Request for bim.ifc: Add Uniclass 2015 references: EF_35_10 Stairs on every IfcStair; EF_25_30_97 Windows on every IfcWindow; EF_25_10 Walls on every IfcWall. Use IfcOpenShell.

First a look at what the model holds.

```python
import ifcopenshell

model = ifcopenshell.open("bim.ifc")
print(model.schema)
print("classifications:", [c.Name for c in model.by_type("IfcClassification")])
for ifc_class in ("IfcDoor", "IfcRoof", "IfcStair", "IfcWall", "IfcWindow"):
    print(ifc_class, len(model.by_type(ifc_class)))
```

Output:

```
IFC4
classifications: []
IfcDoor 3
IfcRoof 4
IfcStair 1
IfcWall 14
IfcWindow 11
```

```python
import ifcopenshell
import ifcopenshell.api.classification

model = ifcopenshell.open("bim.ifc")

system = ifcopenshell.api.classification.add_classification(model, classification="Uniclass 2015")

codes = {
    "IfcStair": ("EF_35_10", "Stairs"),
    "IfcWindow": ("EF_25_30_97", "Windows"),
    "IfcWall": ("EF_25_10", "Walls"),
}
for ifc_class, (code, name) in codes.items():
    products = model.by_type(ifc_class)
    ifcopenshell.api.classification.add_reference(
        model, products=products, classification=system, identification=code, name=name
    )
    print(code, len(products))

model.write("bim_rev.ifc")
```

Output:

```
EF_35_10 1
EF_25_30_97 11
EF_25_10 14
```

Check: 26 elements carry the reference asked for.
